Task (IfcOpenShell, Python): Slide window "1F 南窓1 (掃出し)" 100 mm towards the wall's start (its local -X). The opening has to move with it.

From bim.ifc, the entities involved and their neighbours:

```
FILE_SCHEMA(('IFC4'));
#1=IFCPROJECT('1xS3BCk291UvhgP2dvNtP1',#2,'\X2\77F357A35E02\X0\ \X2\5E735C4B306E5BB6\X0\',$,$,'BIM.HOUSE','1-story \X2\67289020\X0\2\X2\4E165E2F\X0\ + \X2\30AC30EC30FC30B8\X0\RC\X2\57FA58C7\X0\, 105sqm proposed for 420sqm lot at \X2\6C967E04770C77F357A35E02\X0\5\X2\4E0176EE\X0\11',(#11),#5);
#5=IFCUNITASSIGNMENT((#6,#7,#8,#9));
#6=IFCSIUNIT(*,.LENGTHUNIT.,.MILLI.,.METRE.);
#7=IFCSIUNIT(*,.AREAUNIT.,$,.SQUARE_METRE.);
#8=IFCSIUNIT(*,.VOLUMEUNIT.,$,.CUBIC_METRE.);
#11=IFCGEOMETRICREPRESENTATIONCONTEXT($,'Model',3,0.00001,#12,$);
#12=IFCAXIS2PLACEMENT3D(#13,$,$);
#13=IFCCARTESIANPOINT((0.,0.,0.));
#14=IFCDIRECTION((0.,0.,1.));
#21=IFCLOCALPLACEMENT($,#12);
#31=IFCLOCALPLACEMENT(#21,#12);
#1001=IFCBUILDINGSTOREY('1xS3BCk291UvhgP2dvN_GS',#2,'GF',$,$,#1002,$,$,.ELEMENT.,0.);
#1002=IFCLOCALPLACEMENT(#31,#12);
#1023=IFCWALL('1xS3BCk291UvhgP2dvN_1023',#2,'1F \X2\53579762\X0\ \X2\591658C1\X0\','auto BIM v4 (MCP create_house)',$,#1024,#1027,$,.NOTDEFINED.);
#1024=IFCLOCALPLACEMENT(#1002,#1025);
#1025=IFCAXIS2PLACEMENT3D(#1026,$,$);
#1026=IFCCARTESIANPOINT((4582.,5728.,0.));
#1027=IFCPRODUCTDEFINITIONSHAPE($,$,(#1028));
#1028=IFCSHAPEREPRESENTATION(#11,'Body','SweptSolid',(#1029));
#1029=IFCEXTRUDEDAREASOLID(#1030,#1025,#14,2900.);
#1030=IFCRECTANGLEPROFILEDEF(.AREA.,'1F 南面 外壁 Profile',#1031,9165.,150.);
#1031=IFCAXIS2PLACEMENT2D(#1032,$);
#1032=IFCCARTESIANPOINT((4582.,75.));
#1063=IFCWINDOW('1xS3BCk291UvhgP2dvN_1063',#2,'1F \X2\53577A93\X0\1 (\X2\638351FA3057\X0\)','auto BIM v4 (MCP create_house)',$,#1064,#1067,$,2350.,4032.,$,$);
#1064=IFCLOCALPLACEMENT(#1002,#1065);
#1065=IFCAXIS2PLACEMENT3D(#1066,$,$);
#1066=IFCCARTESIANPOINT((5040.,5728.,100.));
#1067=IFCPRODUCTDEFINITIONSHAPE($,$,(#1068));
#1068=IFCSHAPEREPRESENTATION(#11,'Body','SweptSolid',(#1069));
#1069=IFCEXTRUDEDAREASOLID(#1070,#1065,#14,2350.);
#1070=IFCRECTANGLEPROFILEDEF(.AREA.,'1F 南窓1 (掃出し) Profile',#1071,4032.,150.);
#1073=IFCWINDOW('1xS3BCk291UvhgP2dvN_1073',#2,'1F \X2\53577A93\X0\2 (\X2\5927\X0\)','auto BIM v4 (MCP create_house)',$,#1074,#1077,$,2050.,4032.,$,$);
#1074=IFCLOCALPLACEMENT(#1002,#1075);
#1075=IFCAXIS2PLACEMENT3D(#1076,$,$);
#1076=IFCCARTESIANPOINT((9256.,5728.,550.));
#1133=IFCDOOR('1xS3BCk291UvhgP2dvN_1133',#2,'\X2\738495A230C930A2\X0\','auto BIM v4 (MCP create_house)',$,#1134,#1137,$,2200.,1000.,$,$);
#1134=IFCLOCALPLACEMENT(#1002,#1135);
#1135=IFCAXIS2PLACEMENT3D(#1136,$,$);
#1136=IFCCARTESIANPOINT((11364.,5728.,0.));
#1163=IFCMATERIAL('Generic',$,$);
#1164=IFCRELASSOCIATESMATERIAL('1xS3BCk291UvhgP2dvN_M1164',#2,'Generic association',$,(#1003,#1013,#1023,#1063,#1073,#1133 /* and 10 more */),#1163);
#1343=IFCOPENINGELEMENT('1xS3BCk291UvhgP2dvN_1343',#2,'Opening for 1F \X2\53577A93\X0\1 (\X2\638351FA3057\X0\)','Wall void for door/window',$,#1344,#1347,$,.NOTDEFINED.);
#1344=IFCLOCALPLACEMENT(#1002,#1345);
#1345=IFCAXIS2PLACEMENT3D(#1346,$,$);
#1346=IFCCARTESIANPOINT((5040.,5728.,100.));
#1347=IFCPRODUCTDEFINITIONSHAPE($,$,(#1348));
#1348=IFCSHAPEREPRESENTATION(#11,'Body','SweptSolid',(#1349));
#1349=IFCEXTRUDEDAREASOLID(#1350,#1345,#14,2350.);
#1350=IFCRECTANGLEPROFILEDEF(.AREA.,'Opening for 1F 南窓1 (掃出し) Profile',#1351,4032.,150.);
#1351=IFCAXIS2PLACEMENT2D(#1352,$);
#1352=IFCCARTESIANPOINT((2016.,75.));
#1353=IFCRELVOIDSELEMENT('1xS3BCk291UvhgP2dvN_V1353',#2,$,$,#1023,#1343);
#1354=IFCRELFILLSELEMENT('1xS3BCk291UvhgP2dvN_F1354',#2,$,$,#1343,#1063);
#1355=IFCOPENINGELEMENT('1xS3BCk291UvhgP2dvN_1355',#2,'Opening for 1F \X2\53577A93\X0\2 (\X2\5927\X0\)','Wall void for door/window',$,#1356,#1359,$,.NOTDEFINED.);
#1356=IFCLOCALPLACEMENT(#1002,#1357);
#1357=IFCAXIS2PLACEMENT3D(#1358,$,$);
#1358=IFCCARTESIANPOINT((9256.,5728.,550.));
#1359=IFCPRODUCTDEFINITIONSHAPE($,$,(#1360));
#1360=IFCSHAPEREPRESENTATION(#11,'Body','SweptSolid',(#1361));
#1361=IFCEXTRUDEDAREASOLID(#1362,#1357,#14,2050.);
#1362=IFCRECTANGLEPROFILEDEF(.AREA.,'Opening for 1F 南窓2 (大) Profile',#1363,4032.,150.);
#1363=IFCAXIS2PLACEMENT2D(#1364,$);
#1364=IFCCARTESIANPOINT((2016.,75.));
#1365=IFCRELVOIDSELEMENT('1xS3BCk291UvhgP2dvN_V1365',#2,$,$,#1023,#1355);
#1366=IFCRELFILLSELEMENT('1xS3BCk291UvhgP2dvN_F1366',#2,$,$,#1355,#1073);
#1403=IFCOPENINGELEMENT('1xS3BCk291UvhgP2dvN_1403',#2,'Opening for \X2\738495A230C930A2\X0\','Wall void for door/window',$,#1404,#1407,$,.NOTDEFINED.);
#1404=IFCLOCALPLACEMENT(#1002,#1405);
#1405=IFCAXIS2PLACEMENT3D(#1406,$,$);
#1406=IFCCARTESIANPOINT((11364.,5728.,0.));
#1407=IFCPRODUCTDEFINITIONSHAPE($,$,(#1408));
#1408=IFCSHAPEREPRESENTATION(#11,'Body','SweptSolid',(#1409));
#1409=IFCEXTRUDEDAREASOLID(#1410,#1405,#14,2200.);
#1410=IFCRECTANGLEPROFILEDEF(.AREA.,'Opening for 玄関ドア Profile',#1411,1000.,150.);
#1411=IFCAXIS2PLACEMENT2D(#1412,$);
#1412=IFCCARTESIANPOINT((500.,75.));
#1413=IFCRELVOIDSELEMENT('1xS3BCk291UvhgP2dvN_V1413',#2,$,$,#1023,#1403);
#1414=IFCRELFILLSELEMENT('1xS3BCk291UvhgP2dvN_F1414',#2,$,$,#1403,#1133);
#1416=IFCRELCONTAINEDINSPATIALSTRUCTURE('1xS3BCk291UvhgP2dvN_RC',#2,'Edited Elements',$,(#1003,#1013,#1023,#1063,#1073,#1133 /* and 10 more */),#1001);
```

```python
import ifcopenshell
import ifcopenshell.api.geometry
import ifcopenshell.util.placement

model = ifcopenshell.open("bim.ifc")

window = model.by_guid("1xS3BCk291UvhgP2dvN_1063")
opening = window.FillsVoids[0].RelatingOpeningElement
wall = opening.VoidsElements[0].RelatingBuildingElement

wall_matrix = ifcopenshell.util.placement.get_local_placement(wall.ObjectPlacement)
shift = wall_matrix[:3, 0] * -100.0
before = ifcopenshell.util.placement.get_local_placement(window.ObjectPlacement)[:3, 3].copy()

# The window is not placed relative to its opening, so move both.
for product in (opening, window):
    matrix = ifcopenshell.util.placement.get_local_placement(product.ObjectPlacement)
    matrix[:3, 3] += shift
    ifcopenshell.api.geometry.edit_object_placement(model, product=product, matrix=matrix, is_si=False)

after = ifcopenshell.util.placement.get_local_placement(window.ObjectPlacement)[:3, 3]
print("window moved by", (after - before).round(3) + 0.0)

model.write("bim_edited.ifc")
```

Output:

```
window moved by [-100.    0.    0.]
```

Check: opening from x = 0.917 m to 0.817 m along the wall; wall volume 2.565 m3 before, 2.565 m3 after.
